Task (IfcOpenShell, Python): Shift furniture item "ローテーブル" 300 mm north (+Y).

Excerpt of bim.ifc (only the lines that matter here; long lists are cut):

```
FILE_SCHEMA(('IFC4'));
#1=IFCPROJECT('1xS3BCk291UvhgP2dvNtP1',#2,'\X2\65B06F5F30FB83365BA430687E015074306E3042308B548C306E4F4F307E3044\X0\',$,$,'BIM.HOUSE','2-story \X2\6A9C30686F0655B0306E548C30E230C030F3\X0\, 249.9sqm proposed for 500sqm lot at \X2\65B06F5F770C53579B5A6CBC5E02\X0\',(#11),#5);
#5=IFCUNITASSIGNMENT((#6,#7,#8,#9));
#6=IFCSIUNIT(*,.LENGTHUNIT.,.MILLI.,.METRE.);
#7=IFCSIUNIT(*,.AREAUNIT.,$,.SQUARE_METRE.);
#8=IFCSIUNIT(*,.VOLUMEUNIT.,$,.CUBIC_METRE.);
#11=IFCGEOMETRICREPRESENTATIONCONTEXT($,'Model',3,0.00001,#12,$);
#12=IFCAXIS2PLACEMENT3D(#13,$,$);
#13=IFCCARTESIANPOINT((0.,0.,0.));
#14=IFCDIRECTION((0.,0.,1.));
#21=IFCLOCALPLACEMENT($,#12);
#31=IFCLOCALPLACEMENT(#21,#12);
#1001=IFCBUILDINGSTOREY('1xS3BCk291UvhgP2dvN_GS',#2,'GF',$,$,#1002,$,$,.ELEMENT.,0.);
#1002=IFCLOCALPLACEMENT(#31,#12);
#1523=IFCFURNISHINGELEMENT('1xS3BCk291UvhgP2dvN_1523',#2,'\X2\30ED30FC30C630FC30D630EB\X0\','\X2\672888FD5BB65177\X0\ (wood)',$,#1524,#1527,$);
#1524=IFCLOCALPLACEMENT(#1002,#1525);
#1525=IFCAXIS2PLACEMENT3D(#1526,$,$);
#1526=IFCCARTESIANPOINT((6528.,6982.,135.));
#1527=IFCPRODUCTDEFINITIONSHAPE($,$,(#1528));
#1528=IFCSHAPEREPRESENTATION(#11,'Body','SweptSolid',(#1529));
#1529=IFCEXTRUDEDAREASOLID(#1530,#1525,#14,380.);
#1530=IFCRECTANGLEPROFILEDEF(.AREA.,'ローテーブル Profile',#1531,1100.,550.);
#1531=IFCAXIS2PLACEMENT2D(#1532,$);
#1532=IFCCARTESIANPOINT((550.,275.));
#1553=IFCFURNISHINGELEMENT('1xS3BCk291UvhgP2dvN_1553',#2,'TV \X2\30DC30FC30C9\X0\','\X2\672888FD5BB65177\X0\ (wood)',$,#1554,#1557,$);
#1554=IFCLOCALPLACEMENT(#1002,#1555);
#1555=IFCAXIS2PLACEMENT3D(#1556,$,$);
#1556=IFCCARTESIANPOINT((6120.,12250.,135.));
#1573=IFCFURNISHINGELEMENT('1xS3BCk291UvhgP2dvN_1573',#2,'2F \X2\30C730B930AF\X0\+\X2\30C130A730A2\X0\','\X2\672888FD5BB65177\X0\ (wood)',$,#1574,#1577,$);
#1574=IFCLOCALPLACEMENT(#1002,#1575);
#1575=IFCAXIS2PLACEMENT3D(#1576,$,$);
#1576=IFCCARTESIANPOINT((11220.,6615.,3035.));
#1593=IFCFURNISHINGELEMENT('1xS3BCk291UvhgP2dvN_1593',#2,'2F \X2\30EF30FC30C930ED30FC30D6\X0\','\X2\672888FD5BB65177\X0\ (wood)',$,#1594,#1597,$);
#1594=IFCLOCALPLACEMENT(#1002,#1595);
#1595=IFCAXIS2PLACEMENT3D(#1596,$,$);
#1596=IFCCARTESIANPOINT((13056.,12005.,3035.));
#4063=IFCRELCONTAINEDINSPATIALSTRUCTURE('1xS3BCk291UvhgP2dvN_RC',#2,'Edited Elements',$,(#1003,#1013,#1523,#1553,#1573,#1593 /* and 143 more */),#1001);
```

```python
import ifcopenshell
import ifcopenshell.api.geometry
import ifcopenshell.util.placement
import ifcopenshell.util.unit

model = ifcopenshell.open("bim.ifc")
unit_scale = ifcopenshell.util.unit.calculate_unit_scale(model)

item = model.by_id(1523)
matrix = ifcopenshell.util.placement.get_local_placement(item.ObjectPlacement)
matrix[1, 3] += 0.3 / unit_scale
ifcopenshell.api.geometry.edit_object_placement(model, product=item, matrix=matrix, is_si=False)

print(ifcopenshell.util.placement.get_local_placement(item.ObjectPlacement).round(3) + 0.0)

model.write("bim_v2.ifc")
```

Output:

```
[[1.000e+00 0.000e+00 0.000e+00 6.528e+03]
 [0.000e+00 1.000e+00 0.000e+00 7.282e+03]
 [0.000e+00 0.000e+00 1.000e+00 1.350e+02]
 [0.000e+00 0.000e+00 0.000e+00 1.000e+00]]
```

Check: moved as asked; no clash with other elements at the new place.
